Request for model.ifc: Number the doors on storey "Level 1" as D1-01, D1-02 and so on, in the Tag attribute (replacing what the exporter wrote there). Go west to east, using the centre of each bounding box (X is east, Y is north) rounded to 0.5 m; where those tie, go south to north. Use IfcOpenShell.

First a look at what the model holds.

```python
import ifcopenshell
import ifcopenshell.util.element
import ifcopenshell.util.placement

model = ifcopenshell.open("model.ifc")
print(model.schema)
storey = next(s for s in model.by_type("IfcBuildingStorey") if s.Name == "Level 1")
doors = [e for e in ifcopenshell.util.element.get_decomposition(storey) if e.is_a("IfcDoor")]
for e in sorted(doors, key=lambda e: e.id()):
    origin = ifcopenshell.util.placement.get_local_placement(e.ObjectPlacement)[:3, 3]
    print(e.id(), e.Tag, e.Name, origin.round(2) + 0.0, sep=" | ")
```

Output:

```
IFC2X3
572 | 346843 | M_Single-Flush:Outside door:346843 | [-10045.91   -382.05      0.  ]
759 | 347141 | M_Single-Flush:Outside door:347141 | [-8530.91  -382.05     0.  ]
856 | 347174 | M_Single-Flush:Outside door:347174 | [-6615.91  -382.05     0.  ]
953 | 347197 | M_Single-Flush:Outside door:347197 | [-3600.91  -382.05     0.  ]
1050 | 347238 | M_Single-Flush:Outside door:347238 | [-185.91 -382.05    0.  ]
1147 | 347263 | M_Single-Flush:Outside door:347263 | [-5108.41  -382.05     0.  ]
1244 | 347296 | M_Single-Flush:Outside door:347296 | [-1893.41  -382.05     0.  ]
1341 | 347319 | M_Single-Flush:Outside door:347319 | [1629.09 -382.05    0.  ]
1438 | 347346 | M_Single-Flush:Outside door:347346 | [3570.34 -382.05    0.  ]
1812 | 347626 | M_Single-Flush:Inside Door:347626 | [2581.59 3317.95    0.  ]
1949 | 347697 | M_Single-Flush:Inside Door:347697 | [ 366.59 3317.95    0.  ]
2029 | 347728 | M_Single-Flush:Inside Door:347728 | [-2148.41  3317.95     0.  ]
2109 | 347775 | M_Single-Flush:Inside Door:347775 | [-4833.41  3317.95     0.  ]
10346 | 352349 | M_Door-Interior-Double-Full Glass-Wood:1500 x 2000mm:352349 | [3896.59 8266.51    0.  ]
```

```python
import ifcopenshell
import ifcopenshell.geom
import ifcopenshell.util.element
import ifcopenshell.util.shape

model = ifcopenshell.open("model.ifc")
settings = ifcopenshell.geom.settings()
settings.set("use-world-coords", True)


def centre(element):
    shape = ifcopenshell.geom.create_shape(settings, element)
    return ifcopenshell.util.shape.get_bbox_centroid(shape.geometry)


storey = next(s for s in model.by_type("IfcBuildingStorey") if s.Name == "Level 1")
doors = [e for e in ifcopenshell.util.element.get_decomposition(storey) if e.is_a("IfcDoor")]

# Insertion points can sit at a corner or the storey origin, so sort by the geometry (in metres).
centres = {e: centre(e) for e in doors}
doors.sort(key=lambda e: (round(centres[e][0] / 0.5), centres[e][1]))

for i, e in enumerate(doors, start=1):
    number = f"D1-{i:02d}"
    e.Tag = number
    print(e.id(), number)

model.write("model-out.ifc")
```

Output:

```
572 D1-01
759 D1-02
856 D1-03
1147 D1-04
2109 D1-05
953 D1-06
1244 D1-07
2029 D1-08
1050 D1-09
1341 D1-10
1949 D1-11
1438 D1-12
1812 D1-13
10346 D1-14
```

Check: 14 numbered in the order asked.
